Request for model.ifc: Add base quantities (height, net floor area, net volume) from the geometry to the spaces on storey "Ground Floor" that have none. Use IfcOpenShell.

First a look at what the model holds.

```python
import ifcopenshell
import ifcopenshell.util.element
import ifcopenshell.util.unit

model = ifcopenshell.open("model.ifc")
print(model.schema)
for unit_type in ("LENGTHUNIT", "AREAUNIT", "VOLUMEUNIT"):
    print(unit_type, ifcopenshell.util.unit.calculate_unit_scale(model, unit_type))
storey = next(s for s in model.by_type("IfcBuildingStorey") if s.Name == "Ground Floor")
spaces = [e for e in ifcopenshell.util.element.get_decomposition(storey) if e.is_a("IfcSpace")]
for e in sorted(spaces, key=lambda e: e.id()):
    print(e.id(), e.is_a(), e.Name, list(ifcopenshell.util.element.get_psets(e, qtos_only=True)), sep=" | ")
```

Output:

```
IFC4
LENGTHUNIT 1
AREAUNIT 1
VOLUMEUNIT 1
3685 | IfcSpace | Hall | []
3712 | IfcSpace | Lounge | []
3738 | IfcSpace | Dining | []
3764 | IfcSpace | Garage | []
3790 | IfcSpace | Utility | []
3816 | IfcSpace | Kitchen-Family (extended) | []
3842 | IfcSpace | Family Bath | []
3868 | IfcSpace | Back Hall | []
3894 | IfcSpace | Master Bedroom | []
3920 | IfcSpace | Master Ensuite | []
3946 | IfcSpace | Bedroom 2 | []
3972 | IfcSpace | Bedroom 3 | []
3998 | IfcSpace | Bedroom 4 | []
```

```python
import ifcopenshell
import ifcopenshell.api.pset
import ifcopenshell.geom
import ifcopenshell.util.element
import ifcopenshell.util.shape
import ifcopenshell.util.unit

model = ifcopenshell.open("model.ifc")
unit_scale = ifcopenshell.util.unit.calculate_unit_scale(model)
area_scale = ifcopenshell.util.unit.calculate_unit_scale(model, "AREAUNIT")
volume_scale = ifcopenshell.util.unit.calculate_unit_scale(model, "VOLUMEUNIT")
settings = ifcopenshell.geom.settings()

storey = next(s for s in model.by_type("IfcBuildingStorey") if s.Name == "Ground Floor")
spaces = [e for e in ifcopenshell.util.element.get_decomposition(storey) if e.is_a("IfcSpace")]

for e in sorted(spaces, key=lambda e: e.id()):
    if ifcopenshell.util.element.get_psets(e, qtos_only=True, should_inherit=False):
        continue
    # Geometry comes back in metres, in the element's own axes.
    shape = ifcopenshell.geom.create_shape(settings, e)
    values = {
        "Height": ifcopenshell.util.shape.get_z(shape.geometry) / unit_scale,
        "NetFloorArea": ifcopenshell.util.shape.get_footprint_area(shape.geometry) / area_scale,
        "NetVolume": ifcopenshell.util.shape.get_volume(shape.geometry) / volume_scale,
    }
    qto = ifcopenshell.api.pset.add_qto(model, product=e, name="Qto_SpaceBaseQuantities")
    ifcopenshell.api.pset.edit_qto(model, qto=qto, properties=values)
    print(e.id(), {k: round(v, 3) for k, v in values.items()})

model.write("model_updated.ifc")
```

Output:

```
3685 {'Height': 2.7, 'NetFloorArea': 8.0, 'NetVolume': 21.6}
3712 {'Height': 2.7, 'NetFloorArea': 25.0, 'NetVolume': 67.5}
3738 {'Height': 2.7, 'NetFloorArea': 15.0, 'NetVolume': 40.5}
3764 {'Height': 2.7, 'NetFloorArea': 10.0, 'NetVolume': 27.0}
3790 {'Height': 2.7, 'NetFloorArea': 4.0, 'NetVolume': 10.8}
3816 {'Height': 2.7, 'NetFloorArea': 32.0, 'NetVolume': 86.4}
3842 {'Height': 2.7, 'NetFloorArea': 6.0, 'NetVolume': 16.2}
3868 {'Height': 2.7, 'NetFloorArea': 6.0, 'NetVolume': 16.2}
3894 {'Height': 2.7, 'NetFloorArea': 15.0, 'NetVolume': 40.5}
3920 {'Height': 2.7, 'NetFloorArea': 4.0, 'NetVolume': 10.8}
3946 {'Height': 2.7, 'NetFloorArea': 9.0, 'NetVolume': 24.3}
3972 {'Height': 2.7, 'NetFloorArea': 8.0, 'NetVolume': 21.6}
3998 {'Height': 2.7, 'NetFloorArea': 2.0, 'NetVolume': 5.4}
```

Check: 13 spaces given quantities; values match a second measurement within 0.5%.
